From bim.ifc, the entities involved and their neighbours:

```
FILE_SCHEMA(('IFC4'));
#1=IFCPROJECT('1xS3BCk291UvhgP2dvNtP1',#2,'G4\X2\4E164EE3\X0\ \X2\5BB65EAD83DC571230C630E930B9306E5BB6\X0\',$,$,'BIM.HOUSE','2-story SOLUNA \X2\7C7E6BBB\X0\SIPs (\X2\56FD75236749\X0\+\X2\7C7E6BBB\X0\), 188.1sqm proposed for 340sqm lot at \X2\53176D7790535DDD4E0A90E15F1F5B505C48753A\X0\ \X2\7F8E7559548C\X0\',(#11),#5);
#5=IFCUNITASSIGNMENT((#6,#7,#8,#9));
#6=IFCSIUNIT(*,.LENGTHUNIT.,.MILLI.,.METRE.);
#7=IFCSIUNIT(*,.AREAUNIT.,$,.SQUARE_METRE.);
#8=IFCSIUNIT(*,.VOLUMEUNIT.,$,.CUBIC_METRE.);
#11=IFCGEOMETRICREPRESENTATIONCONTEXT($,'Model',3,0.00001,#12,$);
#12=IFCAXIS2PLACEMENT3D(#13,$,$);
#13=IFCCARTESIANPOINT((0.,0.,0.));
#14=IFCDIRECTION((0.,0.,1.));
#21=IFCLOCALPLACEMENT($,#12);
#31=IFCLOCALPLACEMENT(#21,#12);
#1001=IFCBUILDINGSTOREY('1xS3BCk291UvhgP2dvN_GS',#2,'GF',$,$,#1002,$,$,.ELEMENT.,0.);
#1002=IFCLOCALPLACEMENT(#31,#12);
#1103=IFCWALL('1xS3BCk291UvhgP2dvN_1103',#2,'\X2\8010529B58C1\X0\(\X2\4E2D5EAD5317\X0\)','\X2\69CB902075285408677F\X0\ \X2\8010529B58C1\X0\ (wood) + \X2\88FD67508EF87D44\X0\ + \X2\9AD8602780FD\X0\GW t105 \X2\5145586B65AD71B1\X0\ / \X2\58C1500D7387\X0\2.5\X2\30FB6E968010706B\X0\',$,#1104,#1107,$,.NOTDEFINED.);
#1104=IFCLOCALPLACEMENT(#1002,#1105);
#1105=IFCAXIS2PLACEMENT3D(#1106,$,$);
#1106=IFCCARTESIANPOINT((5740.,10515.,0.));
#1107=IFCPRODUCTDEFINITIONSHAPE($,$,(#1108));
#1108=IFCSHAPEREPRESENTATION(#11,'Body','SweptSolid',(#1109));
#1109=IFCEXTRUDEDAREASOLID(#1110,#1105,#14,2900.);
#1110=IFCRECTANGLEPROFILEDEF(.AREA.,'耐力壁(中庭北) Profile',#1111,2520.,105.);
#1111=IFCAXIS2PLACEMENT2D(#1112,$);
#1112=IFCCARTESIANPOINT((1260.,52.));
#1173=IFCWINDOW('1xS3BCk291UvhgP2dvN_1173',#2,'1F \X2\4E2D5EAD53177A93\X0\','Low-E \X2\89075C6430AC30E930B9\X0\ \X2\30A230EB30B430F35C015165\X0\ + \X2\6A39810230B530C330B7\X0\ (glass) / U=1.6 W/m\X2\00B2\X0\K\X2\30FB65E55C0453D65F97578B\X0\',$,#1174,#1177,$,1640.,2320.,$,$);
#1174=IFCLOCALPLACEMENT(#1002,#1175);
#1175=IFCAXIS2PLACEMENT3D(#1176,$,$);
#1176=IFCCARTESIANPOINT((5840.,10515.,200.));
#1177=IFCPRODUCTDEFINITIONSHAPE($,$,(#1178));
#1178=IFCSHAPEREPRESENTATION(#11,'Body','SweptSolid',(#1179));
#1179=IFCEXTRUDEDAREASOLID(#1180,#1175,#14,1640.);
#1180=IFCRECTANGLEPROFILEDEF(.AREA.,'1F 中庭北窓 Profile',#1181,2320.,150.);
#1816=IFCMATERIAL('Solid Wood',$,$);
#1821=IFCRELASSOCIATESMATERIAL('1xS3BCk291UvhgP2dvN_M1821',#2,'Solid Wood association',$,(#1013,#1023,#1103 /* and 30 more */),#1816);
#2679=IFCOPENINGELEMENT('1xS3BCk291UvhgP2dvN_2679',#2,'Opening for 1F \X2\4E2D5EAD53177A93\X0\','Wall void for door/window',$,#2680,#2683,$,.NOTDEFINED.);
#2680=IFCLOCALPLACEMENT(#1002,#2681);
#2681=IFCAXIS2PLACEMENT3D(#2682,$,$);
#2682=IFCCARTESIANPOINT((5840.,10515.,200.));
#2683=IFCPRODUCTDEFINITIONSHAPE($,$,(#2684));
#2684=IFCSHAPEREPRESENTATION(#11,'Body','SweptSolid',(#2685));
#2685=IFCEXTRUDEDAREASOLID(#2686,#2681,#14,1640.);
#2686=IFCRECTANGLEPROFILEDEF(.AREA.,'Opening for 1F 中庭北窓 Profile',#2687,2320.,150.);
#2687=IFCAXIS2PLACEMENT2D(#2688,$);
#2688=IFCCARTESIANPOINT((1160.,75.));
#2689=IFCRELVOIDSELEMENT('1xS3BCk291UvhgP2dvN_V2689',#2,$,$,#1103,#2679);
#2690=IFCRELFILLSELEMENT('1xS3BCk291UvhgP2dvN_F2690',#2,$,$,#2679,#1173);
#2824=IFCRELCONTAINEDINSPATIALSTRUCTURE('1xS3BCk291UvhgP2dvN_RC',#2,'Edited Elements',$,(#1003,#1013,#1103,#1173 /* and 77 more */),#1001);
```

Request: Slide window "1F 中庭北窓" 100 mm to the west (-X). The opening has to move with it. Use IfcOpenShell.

```python
import ifcopenshell
import ifcopenshell.api.geometry
import ifcopenshell.util.placement

model = ifcopenshell.open("bim.ifc")

window = model.by_id(1173)
opening = window.FillsVoids[0].RelatingOpeningElement
wall = opening.VoidsElements[0].RelatingBuildingElement

wall_matrix = ifcopenshell.util.placement.get_local_placement(wall.ObjectPlacement)
shift = wall_matrix[:3, 0] * -100.0
before = ifcopenshell.util.placement.get_local_placement(window.ObjectPlacement)[:3, 3].copy()

# The window is not placed relative to its opening, so move both.
for product in (opening, window):
    matrix = ifcopenshell.util.placement.get_local_placement(product.ObjectPlacement)
    matrix[:3, 3] += shift
    ifcopenshell.api.geometry.edit_object_placement(model, product=product, matrix=matrix, is_si=False)

after = ifcopenshell.util.placement.get_local_placement(window.ObjectPlacement)[:3, 3]
print("window moved by", (after - before).round(3) + 0.0)

model.write("bim_rev.ifc")
```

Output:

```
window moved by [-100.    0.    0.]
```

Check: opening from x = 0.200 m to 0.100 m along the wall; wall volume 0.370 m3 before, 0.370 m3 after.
